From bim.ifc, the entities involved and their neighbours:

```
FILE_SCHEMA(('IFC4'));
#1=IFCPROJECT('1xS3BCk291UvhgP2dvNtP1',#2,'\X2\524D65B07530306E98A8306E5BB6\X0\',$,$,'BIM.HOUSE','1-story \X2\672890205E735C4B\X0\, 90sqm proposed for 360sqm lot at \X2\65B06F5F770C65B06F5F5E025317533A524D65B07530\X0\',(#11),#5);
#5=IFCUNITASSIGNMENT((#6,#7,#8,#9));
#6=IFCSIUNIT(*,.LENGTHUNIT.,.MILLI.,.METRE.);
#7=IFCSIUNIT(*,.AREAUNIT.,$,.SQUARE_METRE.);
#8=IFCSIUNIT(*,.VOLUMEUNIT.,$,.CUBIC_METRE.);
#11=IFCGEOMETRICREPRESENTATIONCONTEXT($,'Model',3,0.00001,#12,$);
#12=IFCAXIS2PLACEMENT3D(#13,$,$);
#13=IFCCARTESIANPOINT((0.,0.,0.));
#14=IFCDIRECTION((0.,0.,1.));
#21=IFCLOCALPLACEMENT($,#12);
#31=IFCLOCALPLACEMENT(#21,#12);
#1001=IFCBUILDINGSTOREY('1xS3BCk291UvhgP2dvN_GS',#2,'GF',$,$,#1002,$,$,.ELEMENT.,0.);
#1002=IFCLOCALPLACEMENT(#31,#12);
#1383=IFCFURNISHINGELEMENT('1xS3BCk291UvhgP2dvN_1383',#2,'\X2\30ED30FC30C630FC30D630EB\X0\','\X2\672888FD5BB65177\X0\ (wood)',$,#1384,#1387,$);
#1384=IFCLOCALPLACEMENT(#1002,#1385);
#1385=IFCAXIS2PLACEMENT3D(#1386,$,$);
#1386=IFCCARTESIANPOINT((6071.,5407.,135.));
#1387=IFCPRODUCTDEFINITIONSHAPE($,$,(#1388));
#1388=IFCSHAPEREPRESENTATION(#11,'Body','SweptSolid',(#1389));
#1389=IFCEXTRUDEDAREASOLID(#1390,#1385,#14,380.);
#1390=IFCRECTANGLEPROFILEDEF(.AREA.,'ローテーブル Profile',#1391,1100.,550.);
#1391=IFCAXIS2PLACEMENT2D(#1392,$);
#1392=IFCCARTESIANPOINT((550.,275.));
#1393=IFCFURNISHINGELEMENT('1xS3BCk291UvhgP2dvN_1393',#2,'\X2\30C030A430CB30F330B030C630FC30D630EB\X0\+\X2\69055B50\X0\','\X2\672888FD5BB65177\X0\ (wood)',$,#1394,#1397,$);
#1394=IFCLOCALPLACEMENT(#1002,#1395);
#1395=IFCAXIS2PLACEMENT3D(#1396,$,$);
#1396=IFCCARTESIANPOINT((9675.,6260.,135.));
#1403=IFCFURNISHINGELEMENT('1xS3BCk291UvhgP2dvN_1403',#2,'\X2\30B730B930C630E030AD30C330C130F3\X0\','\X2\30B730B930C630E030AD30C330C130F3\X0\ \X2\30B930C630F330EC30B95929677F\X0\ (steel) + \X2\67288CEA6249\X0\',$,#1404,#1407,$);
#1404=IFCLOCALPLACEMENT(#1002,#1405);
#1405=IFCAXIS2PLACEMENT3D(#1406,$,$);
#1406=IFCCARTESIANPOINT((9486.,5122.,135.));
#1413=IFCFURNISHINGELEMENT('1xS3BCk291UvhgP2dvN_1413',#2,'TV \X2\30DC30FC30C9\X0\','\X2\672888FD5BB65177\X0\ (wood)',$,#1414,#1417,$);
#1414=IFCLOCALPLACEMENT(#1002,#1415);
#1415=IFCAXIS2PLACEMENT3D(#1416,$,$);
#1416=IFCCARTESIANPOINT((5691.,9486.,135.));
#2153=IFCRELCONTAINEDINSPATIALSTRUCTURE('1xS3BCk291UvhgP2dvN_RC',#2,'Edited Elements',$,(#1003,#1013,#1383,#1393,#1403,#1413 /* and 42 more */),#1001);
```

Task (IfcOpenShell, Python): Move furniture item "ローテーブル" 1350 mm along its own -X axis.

```python
import ifcopenshell
import ifcopenshell.api.geometry
import ifcopenshell.util.placement

model = ifcopenshell.open("bim.ifc")

item = model.by_guid("1xS3BCk291UvhgP2dvN_1383")
matrix = ifcopenshell.util.placement.get_local_placement(item.ObjectPlacement)
matrix[:3, 3] -= matrix[:3, 0] * 1350.0
ifcopenshell.api.geometry.edit_object_placement(model, product=item, matrix=matrix, is_si=False)

print(ifcopenshell.util.placement.get_local_placement(item.ObjectPlacement).round(3) + 0.0)

model.write("bim_v2.ifc")
```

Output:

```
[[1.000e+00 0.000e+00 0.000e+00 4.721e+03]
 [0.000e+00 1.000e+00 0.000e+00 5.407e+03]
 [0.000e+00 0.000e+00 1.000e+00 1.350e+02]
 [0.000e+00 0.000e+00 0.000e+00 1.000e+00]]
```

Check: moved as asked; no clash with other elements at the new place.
